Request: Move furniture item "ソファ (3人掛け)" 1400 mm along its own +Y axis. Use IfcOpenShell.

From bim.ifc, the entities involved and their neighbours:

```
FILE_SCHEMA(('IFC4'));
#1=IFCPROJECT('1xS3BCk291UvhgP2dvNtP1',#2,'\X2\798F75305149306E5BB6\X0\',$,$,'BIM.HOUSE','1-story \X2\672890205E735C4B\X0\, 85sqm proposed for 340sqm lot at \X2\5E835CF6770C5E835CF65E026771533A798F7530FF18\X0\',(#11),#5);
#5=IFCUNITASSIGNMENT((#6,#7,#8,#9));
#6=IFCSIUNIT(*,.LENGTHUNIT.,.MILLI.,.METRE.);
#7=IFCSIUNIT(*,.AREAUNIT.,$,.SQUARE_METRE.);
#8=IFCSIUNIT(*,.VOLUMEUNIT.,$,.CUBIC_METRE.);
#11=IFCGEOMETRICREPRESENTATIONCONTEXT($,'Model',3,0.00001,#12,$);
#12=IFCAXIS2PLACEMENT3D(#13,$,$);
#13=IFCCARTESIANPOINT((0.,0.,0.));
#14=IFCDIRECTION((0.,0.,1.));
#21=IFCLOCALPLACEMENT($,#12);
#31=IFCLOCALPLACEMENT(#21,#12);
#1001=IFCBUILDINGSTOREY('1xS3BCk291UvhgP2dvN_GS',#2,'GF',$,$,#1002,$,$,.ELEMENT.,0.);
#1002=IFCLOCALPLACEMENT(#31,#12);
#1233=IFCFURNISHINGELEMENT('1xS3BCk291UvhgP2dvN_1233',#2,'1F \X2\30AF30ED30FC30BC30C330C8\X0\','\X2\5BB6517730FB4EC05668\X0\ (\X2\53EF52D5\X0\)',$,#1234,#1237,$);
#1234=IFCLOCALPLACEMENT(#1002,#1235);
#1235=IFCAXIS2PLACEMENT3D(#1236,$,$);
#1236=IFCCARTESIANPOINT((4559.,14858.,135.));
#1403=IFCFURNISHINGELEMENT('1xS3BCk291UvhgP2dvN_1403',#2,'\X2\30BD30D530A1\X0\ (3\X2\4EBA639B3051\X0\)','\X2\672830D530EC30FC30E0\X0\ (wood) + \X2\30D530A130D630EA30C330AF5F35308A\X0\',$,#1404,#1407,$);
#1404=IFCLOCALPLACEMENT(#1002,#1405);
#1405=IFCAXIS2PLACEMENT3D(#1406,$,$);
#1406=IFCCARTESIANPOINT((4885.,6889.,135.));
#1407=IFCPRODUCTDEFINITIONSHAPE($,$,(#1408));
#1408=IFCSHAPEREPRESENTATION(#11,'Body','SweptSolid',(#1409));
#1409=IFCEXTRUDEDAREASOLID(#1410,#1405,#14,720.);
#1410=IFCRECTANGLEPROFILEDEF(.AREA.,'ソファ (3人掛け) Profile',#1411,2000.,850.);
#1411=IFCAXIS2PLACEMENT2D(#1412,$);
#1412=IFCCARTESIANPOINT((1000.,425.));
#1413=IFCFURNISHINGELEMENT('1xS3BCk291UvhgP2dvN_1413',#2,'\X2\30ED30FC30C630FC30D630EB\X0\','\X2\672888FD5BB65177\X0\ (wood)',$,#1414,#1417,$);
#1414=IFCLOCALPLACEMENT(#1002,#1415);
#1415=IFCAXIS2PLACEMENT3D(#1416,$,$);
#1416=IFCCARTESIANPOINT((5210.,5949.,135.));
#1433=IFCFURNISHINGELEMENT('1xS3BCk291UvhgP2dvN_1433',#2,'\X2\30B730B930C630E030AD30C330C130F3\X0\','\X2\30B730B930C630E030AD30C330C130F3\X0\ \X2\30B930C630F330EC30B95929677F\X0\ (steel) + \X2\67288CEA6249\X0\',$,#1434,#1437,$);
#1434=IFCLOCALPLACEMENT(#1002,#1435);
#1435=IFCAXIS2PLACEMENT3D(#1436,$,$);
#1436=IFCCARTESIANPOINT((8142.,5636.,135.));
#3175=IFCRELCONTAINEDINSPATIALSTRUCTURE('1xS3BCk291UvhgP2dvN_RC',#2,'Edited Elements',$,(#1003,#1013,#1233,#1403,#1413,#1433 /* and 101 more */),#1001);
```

```python
import ifcopenshell
import ifcopenshell.api.geometry
import ifcopenshell.util.placement
import ifcopenshell.util.unit

model = ifcopenshell.open("bim.ifc")
unit_scale = ifcopenshell.util.unit.calculate_unit_scale(model)

item = model.by_id(1403)
matrix = ifcopenshell.util.placement.get_local_placement(item.ObjectPlacement)
matrix[:3, 3] += matrix[:3, 1] * 1.4 / unit_scale
ifcopenshell.api.geometry.edit_object_placement(model, product=item, matrix=matrix, is_si=False)

print(ifcopenshell.util.placement.get_local_placement(item.ObjectPlacement).round(3) + 0.0)

model.write("bim-out.ifc")
```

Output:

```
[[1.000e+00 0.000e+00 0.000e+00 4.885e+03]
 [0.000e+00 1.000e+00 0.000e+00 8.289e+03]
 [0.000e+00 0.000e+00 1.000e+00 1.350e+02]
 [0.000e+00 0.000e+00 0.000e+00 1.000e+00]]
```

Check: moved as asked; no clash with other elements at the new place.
